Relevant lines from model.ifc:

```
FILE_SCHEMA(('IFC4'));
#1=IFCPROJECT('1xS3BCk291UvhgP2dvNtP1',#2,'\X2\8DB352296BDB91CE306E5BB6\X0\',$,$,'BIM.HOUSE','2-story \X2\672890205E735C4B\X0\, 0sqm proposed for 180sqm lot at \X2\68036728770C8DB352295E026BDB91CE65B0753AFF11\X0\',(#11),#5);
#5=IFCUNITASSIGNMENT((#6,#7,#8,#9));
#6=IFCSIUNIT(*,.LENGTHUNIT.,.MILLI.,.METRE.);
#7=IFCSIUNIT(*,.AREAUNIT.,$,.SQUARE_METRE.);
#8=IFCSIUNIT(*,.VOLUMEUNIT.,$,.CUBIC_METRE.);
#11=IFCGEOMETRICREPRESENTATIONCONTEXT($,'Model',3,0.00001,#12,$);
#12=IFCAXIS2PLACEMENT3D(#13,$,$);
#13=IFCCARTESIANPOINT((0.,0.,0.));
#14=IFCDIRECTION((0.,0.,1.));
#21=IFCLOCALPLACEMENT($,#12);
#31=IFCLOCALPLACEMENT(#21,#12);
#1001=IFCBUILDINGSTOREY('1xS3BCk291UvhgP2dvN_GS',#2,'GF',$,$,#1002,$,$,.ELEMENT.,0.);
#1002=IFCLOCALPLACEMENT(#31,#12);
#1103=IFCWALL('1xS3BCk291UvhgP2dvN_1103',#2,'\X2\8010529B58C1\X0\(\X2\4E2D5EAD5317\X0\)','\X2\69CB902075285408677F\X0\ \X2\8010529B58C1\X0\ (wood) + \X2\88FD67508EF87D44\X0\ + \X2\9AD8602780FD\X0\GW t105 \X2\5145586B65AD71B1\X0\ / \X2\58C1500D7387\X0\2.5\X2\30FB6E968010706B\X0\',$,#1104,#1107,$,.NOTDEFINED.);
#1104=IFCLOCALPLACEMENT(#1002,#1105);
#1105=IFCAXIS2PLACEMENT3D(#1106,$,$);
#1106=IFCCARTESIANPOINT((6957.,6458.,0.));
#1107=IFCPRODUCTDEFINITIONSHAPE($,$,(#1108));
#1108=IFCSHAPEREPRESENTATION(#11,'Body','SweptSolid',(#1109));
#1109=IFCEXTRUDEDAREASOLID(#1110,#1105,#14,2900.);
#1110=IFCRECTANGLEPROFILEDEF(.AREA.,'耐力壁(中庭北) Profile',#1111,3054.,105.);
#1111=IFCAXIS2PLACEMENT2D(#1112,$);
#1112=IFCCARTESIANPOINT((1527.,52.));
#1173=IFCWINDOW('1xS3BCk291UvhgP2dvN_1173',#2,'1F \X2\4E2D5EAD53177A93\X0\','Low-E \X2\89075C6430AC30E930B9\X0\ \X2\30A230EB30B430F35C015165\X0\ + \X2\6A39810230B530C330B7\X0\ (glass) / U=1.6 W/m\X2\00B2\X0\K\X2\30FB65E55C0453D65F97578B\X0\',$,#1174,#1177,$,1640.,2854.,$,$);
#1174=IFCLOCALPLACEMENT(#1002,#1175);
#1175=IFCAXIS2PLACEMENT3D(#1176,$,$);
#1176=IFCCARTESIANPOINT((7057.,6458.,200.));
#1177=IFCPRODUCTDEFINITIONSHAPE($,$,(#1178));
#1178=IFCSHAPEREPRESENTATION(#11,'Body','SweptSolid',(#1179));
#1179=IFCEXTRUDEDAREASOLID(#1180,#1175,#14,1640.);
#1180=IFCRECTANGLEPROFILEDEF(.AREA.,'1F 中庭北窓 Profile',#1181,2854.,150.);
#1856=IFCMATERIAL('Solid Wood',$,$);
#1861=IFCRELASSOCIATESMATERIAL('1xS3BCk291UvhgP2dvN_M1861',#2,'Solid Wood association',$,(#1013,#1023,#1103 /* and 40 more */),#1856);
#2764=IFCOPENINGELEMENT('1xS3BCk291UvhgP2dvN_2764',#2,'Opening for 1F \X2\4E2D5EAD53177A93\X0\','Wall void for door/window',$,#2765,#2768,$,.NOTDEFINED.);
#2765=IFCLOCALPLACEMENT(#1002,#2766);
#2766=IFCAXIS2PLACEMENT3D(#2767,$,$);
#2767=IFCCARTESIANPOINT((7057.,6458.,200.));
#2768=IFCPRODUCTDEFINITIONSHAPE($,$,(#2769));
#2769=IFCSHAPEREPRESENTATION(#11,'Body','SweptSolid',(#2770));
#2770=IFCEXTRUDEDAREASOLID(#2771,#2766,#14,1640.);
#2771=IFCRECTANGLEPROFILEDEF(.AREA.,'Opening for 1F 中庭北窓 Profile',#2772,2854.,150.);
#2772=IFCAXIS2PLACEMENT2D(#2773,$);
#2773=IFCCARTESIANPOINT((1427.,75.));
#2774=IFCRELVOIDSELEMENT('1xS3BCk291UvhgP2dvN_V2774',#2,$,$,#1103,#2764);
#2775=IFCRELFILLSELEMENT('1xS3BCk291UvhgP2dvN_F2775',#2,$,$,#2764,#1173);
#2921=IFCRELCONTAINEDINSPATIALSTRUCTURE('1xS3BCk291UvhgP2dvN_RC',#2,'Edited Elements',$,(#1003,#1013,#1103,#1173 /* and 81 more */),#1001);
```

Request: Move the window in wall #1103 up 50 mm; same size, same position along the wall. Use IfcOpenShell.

```python
import numpy as np
import ifcopenshell
import ifcopenshell.api.geometry
import ifcopenshell.util.placement
import ifcopenshell.util.unit

model = ifcopenshell.open("model.ifc")
unit_scale = ifcopenshell.util.unit.calculate_unit_scale(model)

window = model.by_guid("1xS3BCk291UvhgP2dvN_1173")
opening = window.FillsVoids[0].RelatingOpeningElement
dz = 0.05 / unit_scale

shift = np.array([0.0, 0.0, dz])
# The window is not placed relative to its opening, so move both.
for product in (opening, window):
    matrix = ifcopenshell.util.placement.get_local_placement(product.ObjectPlacement)
    matrix[:3, 3] += shift
    ifcopenshell.api.geometry.edit_object_placement(model, product=product, matrix=matrix, is_si=False)

print(f"moved by {dz * unit_scale:+.3f} m")

model.write("model_edited.ifc")
```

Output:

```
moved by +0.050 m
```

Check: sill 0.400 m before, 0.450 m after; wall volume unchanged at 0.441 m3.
